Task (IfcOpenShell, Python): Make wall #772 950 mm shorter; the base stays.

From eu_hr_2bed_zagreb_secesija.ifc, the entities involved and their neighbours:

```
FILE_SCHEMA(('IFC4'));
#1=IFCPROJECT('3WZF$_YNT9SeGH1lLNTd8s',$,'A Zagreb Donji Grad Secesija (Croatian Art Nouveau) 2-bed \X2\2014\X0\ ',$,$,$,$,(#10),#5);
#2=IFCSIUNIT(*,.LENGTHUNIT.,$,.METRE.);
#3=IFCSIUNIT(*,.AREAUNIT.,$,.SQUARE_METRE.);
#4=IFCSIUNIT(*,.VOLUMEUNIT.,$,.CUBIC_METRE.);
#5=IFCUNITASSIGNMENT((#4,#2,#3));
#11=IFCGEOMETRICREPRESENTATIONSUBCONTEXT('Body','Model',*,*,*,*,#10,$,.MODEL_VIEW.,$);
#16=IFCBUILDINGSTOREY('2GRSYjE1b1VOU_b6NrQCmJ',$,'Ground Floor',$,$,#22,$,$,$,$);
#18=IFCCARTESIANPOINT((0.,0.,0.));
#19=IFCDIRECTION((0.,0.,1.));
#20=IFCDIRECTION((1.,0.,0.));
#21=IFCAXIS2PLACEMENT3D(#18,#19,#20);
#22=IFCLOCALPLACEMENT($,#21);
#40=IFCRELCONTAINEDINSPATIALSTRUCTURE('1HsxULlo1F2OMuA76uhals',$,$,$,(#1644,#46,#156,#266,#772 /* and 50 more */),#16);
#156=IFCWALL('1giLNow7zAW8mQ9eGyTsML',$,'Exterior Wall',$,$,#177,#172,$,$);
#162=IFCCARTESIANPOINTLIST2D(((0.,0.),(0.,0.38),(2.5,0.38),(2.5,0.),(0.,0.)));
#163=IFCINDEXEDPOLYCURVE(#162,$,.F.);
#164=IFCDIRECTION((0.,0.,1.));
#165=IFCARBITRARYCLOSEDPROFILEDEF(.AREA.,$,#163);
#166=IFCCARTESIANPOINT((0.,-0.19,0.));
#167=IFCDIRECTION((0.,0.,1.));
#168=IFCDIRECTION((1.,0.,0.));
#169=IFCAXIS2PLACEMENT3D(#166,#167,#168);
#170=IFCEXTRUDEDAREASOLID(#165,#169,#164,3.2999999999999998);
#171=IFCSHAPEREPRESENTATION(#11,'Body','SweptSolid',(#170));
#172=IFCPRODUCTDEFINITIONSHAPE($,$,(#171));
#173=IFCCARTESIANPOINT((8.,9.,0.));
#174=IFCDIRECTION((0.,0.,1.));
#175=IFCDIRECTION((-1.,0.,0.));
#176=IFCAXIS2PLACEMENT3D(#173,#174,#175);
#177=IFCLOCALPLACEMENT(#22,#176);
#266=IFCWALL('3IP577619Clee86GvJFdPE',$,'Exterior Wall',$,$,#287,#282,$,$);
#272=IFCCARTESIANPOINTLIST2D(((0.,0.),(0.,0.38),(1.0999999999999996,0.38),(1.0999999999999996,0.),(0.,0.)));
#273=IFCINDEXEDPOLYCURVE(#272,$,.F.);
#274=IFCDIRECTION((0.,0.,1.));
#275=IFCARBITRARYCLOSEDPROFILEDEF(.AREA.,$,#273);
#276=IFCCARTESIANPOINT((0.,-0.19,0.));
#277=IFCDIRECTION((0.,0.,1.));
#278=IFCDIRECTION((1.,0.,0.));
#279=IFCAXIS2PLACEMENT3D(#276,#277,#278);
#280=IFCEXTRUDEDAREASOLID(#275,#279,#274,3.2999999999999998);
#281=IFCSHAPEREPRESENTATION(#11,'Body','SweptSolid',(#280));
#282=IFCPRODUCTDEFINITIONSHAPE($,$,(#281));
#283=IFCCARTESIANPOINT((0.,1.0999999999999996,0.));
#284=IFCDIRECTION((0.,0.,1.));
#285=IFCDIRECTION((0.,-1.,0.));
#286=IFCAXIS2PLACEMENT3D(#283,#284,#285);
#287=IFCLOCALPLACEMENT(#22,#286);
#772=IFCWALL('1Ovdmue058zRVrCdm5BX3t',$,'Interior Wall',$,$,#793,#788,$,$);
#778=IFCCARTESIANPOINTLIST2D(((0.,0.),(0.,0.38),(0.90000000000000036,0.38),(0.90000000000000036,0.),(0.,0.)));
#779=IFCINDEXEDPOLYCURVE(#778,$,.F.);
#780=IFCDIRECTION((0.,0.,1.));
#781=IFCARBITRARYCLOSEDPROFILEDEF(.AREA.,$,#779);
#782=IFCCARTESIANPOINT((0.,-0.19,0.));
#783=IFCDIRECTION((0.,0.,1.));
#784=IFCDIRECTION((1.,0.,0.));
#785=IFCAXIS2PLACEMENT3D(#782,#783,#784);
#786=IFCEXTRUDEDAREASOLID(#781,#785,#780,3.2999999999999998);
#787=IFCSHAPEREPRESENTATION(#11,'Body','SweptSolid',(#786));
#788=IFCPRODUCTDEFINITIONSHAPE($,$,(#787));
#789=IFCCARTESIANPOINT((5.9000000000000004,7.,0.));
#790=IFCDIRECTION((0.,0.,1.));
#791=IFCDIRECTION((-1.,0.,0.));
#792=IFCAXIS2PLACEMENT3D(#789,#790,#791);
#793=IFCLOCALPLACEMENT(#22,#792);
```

```python
import ifcopenshell
import ifcopenshell.geom
import ifcopenshell.util.representation
import ifcopenshell.util.shape

model = ifcopenshell.open("eu_hr_2bed_zagreb_secesija.ifc")
settings = ifcopenshell.geom.settings()


def volume(element):
    """Net volume in cubic metres, openings subtracted."""
    shape = ifcopenshell.geom.create_shape(settings, element)
    return ifcopenshell.util.shape.get_volume(shape.geometry)


wall = model.by_guid("1Ovdmue058zRVrCdm5BX3t")
before = volume(wall)

body = ifcopenshell.util.representation.get_representation(wall, "Model", "Body")
solid = body.Items[0]
old_height = solid.Depth
solid.Depth -= 0.95
after = volume(wall)

print(f"height {old_height:g} -> {solid.Depth:g}, volume {before:.3f} -> {after:.3f} m3")

model.write("eu_hr_2bed_zagreb_secesija_rev.ifc")
```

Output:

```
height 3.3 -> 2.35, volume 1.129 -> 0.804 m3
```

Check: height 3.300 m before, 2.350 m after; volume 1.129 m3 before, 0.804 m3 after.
